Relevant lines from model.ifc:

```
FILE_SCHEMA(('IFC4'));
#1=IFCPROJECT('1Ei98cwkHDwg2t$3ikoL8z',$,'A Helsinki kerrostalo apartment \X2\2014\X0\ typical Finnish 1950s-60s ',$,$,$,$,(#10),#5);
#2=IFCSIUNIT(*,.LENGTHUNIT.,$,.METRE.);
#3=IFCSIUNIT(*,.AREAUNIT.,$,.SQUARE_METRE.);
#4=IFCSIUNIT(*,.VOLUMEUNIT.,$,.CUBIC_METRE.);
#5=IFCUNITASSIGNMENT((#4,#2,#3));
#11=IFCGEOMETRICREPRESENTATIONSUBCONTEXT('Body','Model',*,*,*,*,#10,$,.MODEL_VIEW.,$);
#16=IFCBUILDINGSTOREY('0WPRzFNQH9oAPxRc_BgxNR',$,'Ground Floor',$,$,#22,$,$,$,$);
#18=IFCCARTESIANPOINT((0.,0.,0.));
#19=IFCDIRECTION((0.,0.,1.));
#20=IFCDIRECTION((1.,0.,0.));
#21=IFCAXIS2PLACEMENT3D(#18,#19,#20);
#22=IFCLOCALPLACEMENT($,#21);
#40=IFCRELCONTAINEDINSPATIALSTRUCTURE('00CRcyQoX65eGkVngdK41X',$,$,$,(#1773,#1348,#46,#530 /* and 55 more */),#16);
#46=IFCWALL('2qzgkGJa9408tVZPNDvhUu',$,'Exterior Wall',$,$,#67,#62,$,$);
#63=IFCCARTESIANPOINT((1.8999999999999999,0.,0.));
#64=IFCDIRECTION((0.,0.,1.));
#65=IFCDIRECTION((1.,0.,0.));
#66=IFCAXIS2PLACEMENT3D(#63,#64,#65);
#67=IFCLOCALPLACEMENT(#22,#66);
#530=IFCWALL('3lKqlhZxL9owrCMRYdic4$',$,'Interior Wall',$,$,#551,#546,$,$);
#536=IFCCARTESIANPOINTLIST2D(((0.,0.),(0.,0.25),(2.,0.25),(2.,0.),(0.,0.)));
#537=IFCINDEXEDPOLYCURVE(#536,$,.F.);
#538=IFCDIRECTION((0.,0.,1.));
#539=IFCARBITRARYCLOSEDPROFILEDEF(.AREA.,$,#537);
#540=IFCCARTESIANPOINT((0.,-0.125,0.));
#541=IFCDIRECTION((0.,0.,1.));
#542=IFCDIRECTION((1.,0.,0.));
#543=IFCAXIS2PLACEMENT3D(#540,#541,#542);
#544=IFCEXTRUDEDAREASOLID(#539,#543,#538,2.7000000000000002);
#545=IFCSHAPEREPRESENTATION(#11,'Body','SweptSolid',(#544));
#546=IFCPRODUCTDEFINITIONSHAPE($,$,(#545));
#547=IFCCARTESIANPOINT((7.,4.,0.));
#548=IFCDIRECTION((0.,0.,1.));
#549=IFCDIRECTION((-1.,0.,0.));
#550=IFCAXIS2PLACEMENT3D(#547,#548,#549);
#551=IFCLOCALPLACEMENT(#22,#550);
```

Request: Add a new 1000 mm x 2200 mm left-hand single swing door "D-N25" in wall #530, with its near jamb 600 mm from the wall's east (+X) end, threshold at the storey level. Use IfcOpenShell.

```python
import numpy as np
import ifcopenshell
import ifcopenshell.api.feature
import ifcopenshell.api.geometry
import ifcopenshell.api.root
import ifcopenshell.api.spatial
import ifcopenshell.geom
import ifcopenshell.util.element
import ifcopenshell.util.placement
import ifcopenshell.util.representation
import ifcopenshell.util.shape
import ifcopenshell.util.unit

model = ifcopenshell.open("model.ifc")
unit_scale = ifcopenshell.util.unit.calculate_unit_scale(model)
settings = ifcopenshell.geom.settings()


def volume(element):
    """Net volume in cubic metres, openings subtracted."""
    shape = ifcopenshell.geom.create_shape(settings, element)
    return ifcopenshell.util.shape.get_volume(shape.geometry)


wall = model.by_guid("3lKqlhZxL9owrCMRYdic4$")
storey = ifcopenshell.util.element.get_container(wall, ifc_class="IfcBuildingStorey")
context = ifcopenshell.util.representation.get_context(model, "Model", "Body", "MODEL_VIEW")
before = volume(wall)

width, height, from_end, sill = 1, 2.2, 0.6, 0.0  # metres

# The wall runs along its own X axis, and the end named is its -X end.
wall_shape = ifcopenshell.geom.create_shape(settings, wall)
x, y, z = ifcopenshell.util.shape.get_vertices(wall_shape.geometry).T
start = x.min() + from_end
face, thickness = float(y.min()), float(y.max() - y.min())
wall_matrix = ifcopenshell.util.placement.get_local_placement(wall.ObjectPlacement)
level = ifcopenshell.util.placement.get_local_placement(storey.ObjectPlacement)[2, 3]


def in_wall(x, y):
    """Placement at x, y metres in the wall's axes, at sill height."""
    matrix = wall_matrix.copy()
    matrix[:, 3] = wall_matrix @ np.array([x / unit_scale, y / unit_scale, 0.0, 1.0])
    matrix[2, 3] = level + sill / unit_scale
    return matrix


# Opening: a box that overshoots both wall faces by 50 mm.
opening = ifcopenshell.api.root.create_entity(model, ifc_class="IfcOpeningElement", predefined_type="OPENING")
box = ifcopenshell.api.geometry.add_wall_representation(
    model, context=context, length=width, height=height, thickness=thickness + 0.1
)
ifcopenshell.api.geometry.assign_representation(model, product=opening, representation=box)
ifcopenshell.api.geometry.edit_object_placement(model, product=opening, matrix=in_wall(start, face - 0.05), is_si=False)
ifcopenshell.api.feature.add_feature(model, feature=opening, element=wall)

door = ifcopenshell.api.root.create_entity(model, ifc_class="IfcDoor", name="D-N25", predefined_type="DOOR")
door.OverallWidth, door.OverallHeight = width / unit_scale, height / unit_scale
door.OperationType = "SINGLE_SWING_LEFT"
body = ifcopenshell.api.geometry.add_door_representation(
    model,
    context=context,
    overall_width=door.OverallWidth,
    overall_height=door.OverallHeight,
    operation_type="SINGLE_SWING_LEFT",
    lining_properties={"LiningDepth": thickness / unit_scale, "ThresholdDepth": thickness / unit_scale},
)
ifcopenshell.api.geometry.assign_representation(model, product=door, representation=body)
ifcopenshell.api.spatial.assign_container(model, products=[door], relating_structure=storey)
ifcopenshell.api.feature.add_filling(model, opening=opening, element=door)

# The lining spans the wall, so the door starts at the wall face.
ifcopenshell.api.geometry.edit_object_placement(model, product=door, matrix=in_wall(start, face), is_si=False)

after = volume(wall)

print(f"wall volume {before:.3f} -> {after:.3f} m3")

model.write("model_v2.ifc")
```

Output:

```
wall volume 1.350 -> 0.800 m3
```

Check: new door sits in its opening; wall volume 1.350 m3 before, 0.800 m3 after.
